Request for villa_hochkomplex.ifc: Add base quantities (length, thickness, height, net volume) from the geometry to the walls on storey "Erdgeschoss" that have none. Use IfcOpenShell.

First a look at what the model holds.

```python
import ifcopenshell
import ifcopenshell.util.element
import ifcopenshell.util.unit

model = ifcopenshell.open("villa_hochkomplex.ifc")
print(model.schema)
for unit_type in ("LENGTHUNIT", "AREAUNIT", "VOLUMEUNIT"):
    print(unit_type, ifcopenshell.util.unit.calculate_unit_scale(model, unit_type))
storey = next(s for s in model.by_type("IfcBuildingStorey") if s.Name == "Erdgeschoss")
walls = [e for e in ifcopenshell.util.element.get_decomposition(storey) if e.is_a("IfcWall")]
for e in sorted(walls, key=lambda e: e.id()):
    print(e.id(), e.is_a(), e.Name, list(ifcopenshell.util.element.get_psets(e, qtos_only=True)), sep=" | ")
```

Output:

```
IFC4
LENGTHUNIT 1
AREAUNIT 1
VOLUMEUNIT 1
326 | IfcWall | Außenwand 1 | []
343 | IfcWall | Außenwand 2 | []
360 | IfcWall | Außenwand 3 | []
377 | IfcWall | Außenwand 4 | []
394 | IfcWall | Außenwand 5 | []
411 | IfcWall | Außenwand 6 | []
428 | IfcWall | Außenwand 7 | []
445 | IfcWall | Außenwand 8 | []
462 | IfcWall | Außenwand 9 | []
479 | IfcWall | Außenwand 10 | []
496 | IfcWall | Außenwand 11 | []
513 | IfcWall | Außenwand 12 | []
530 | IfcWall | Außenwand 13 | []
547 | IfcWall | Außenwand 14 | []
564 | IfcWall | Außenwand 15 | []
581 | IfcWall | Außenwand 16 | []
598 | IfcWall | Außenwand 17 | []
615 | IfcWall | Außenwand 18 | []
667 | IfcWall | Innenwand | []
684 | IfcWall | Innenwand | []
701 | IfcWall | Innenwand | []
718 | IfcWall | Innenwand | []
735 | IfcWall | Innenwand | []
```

```python
import ifcopenshell
import ifcopenshell.api.pset
import ifcopenshell.geom
import ifcopenshell.util.element
import ifcopenshell.util.shape
import ifcopenshell.util.unit

model = ifcopenshell.open("villa_hochkomplex.ifc")
unit_scale = ifcopenshell.util.unit.calculate_unit_scale(model)
volume_scale = ifcopenshell.util.unit.calculate_unit_scale(model, "VOLUMEUNIT")
settings = ifcopenshell.geom.settings()

storey = next(s for s in model.by_type("IfcBuildingStorey") if s.Name == "Erdgeschoss")
walls = [e for e in ifcopenshell.util.element.get_decomposition(storey) if e.is_a("IfcWall")]

for e in sorted(walls, key=lambda e: e.id()):
    if ifcopenshell.util.element.get_psets(e, qtos_only=True, should_inherit=False):
        continue
    # Geometry comes back in metres, in the element's own axes.
    shape = ifcopenshell.geom.create_shape(settings, e)
    values = {
        "Length": ifcopenshell.util.shape.get_x(shape.geometry) / unit_scale,
        "Width": ifcopenshell.util.shape.get_y(shape.geometry) / unit_scale,
        "Height": ifcopenshell.util.shape.get_z(shape.geometry) / unit_scale,
        "NetVolume": ifcopenshell.util.shape.get_volume(shape.geometry) / volume_scale,
    }
    qto = ifcopenshell.api.pset.add_qto(model, product=e, name="Qto_WallBaseQuantities")
    ifcopenshell.api.pset.edit_qto(model, qto=qto, properties=values)
    print(e.id(), {k: round(v, 3) for k, v in values.items()})

model.write("villa_hochkomplex_edited.ifc")
```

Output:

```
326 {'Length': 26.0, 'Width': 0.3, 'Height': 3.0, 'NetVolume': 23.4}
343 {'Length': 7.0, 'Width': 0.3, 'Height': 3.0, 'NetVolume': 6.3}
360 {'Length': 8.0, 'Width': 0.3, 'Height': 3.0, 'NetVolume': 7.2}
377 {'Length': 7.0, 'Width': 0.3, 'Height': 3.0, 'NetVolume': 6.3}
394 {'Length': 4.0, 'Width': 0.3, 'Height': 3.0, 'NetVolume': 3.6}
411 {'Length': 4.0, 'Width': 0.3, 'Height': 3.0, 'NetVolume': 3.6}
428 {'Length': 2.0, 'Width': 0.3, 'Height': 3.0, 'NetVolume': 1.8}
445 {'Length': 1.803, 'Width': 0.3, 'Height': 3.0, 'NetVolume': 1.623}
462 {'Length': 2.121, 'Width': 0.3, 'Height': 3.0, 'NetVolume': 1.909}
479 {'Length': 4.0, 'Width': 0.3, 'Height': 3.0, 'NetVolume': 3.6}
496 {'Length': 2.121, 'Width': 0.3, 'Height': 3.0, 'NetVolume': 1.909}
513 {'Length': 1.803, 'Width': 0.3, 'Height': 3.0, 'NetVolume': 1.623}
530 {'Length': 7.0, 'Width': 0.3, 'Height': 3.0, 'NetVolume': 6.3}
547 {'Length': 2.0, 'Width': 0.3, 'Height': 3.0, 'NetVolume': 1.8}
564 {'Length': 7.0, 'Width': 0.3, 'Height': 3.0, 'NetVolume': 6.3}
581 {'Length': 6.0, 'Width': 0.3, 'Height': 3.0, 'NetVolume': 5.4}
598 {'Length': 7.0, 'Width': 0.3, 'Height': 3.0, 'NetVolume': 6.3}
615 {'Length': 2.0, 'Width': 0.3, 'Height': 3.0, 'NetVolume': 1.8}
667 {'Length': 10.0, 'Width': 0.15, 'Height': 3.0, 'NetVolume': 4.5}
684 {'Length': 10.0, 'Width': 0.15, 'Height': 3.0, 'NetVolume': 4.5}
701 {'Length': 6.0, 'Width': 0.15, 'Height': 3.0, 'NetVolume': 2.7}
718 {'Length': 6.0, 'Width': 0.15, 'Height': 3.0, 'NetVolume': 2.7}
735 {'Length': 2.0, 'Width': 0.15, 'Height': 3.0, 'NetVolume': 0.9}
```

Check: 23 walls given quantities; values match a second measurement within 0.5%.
